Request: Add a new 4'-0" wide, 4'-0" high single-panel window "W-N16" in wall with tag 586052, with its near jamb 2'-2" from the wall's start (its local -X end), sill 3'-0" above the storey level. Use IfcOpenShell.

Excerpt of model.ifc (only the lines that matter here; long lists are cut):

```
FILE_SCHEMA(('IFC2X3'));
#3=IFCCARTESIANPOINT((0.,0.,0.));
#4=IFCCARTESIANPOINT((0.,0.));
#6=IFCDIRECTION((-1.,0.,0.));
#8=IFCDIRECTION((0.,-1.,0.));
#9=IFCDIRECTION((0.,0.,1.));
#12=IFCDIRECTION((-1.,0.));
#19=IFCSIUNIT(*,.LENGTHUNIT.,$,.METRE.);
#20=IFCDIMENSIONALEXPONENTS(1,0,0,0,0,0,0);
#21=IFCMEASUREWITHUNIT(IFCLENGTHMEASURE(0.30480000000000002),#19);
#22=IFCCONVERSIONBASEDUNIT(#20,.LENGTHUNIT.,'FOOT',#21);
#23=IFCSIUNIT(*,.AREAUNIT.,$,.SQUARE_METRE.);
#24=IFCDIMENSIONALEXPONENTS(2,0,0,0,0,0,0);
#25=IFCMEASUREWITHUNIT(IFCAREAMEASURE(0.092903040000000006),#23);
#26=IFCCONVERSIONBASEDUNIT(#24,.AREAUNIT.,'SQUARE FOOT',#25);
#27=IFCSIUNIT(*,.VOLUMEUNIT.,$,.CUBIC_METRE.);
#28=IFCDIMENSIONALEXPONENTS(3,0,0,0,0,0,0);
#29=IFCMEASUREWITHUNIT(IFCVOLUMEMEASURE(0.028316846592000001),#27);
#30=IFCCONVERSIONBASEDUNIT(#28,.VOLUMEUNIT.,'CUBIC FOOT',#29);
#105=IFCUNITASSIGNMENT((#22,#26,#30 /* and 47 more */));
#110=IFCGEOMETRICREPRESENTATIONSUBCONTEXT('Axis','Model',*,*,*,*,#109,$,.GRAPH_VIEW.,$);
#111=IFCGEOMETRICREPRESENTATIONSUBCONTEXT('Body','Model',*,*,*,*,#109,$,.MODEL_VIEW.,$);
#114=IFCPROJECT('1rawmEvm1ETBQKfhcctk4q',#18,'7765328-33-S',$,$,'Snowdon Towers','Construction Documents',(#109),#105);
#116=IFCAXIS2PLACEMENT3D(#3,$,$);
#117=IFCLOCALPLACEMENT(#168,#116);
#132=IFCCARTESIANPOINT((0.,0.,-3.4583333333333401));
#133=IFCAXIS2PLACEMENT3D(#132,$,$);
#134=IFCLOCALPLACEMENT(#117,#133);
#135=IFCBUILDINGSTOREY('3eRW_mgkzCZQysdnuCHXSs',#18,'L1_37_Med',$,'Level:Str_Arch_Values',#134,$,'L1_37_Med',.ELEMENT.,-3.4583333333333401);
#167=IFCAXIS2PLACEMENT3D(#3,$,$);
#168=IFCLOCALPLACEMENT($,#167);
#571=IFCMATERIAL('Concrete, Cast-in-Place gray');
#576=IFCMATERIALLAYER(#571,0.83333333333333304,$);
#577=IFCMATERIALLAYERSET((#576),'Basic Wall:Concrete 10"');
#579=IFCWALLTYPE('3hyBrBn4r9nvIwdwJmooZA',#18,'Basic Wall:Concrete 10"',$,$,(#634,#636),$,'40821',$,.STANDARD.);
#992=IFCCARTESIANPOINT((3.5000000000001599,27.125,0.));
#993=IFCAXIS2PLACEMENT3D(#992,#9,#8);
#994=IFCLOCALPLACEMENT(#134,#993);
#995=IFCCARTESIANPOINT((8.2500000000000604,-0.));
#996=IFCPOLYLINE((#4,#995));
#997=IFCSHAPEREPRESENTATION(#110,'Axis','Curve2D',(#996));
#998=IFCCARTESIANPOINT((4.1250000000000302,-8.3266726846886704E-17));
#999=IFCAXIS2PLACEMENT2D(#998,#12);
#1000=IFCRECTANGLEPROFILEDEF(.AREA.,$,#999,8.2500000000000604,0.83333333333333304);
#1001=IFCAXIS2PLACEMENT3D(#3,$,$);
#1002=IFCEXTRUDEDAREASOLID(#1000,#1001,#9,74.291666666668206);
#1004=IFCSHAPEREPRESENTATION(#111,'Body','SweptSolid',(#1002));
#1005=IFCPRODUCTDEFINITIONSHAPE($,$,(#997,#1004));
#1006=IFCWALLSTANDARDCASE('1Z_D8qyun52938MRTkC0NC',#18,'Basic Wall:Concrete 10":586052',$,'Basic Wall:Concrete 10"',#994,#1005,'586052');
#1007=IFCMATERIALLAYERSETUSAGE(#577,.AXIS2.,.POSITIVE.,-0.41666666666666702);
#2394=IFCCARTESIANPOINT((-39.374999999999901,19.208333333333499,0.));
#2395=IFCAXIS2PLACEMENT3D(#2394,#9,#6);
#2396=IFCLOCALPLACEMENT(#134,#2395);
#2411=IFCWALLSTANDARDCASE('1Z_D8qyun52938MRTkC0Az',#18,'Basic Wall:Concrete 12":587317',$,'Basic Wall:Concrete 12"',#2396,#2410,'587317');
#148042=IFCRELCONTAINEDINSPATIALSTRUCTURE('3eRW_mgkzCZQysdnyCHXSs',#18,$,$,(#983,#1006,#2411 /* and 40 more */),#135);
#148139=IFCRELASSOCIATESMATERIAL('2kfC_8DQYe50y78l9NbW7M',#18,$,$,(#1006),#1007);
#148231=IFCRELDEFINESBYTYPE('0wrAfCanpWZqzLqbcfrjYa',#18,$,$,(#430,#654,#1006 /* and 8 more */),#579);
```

```python
import numpy as np
import ifcopenshell
import ifcopenshell.api.feature
import ifcopenshell.api.geometry
import ifcopenshell.api.root
import ifcopenshell.api.spatial
import ifcopenshell.api.type
import ifcopenshell.geom
import ifcopenshell.util.element
import ifcopenshell.util.placement
import ifcopenshell.util.representation
import ifcopenshell.util.shape
import ifcopenshell.util.unit

model = ifcopenshell.open("model.ifc")
unit_scale = ifcopenshell.util.unit.calculate_unit_scale(model)
settings = ifcopenshell.geom.settings()


def volume(element):
    """Net volume in cubic metres, openings subtracted."""
    shape = ifcopenshell.geom.create_shape(settings, element)
    return ifcopenshell.util.shape.get_volume(shape.geometry)


wall = model.by_id(1006)
storey = ifcopenshell.util.element.get_container(wall, ifc_class="IfcBuildingStorey")
context = ifcopenshell.util.representation.get_context(model, "Model", "Body", "MODEL_VIEW")
before = volume(wall)

width, height, from_end, sill = 1.2192, 1.2192, 0.6604, 0.9144  # metres

# The wall runs along its own X axis, and the end named is its -X end.
wall_shape = ifcopenshell.geom.create_shape(settings, wall)
x, y, z = ifcopenshell.util.shape.get_vertices(wall_shape.geometry).T
start = x.min() + from_end
face, thickness = float(y.min()), float(y.max() - y.min())
wall_matrix = ifcopenshell.util.placement.get_local_placement(wall.ObjectPlacement)
level = ifcopenshell.util.placement.get_local_placement(storey.ObjectPlacement)[2, 3]


def in_wall(x, y):
    """Placement at x, y metres in the wall's axes, at sill height."""
    matrix = wall_matrix.copy()
    matrix[:, 3] = wall_matrix @ np.array([x / unit_scale, y / unit_scale, 0.0, 1.0])
    matrix[2, 3] = level + sill / unit_scale
    return matrix


# Opening: a box that overshoots both wall faces by 50 mm.
opening = ifcopenshell.api.root.create_entity(model, ifc_class="IfcOpeningElement")
box = ifcopenshell.api.geometry.add_wall_representation(
    model, context=context, length=width, height=height, thickness=thickness + 0.1
)
ifcopenshell.api.geometry.assign_representation(model, product=opening, representation=box)
ifcopenshell.api.geometry.edit_object_placement(model, product=opening, matrix=in_wall(start, face - 0.05), is_si=False)
ifcopenshell.api.feature.add_feature(model, feature=opening, element=wall)

window = ifcopenshell.api.root.create_entity(model, ifc_class="IfcWindow", name="W-N16")
window.OverallWidth, window.OverallHeight = width / unit_scale, height / unit_scale
body = ifcopenshell.api.geometry.add_window_representation(
    model,
    context=context,
    overall_width=window.OverallWidth,
    overall_height=window.OverallHeight,
    partition_type="SINGLE_PANEL",
)
ifcopenshell.api.geometry.assign_representation(model, product=window, representation=body)
ifcopenshell.api.spatial.assign_container(model, products=[window], relating_structure=storey)
fills = ifcopenshell.api.feature.add_filling(model, opening=opening, element=window)
fills.OwnerHistory = window.OwnerHistory  # required in IFC2X3

# IFC2X3 keeps the operation on the window style.
style = ifcopenshell.api.root.create_entity(model, ifc_class="IfcWindowStyle", name="W-N16")
style.OperationType, style.ConstructionType = "SINGLE_PANEL", "NOTDEFINED"
style.ParameterTakesPrecedence = style.Sizeable = False
ifcopenshell.api.type.assign_type(model, related_objects=[window], relating_type=style)

# Centre the window in the wall's thickness.
ifcopenshell.api.geometry.edit_object_placement(model, product=window, matrix=in_wall(start, face), is_si=False)
window_shape = ifcopenshell.geom.create_shape(settings, window)
depth = ifcopenshell.util.shape.get_vertices(window_shape.geometry)[:, 1]
offset = face + thickness / 2 - (depth.min() + depth.max()) / 2
ifcopenshell.api.geometry.edit_object_placement(model, product=window, matrix=in_wall(start, offset), is_si=False)

after = volume(wall)

print(f"wall volume {before:.3f} -> {after:.3f} m3")

model.write("model_v2.ifc")
```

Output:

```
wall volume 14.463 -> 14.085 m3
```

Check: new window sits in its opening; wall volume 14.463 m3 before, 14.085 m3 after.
